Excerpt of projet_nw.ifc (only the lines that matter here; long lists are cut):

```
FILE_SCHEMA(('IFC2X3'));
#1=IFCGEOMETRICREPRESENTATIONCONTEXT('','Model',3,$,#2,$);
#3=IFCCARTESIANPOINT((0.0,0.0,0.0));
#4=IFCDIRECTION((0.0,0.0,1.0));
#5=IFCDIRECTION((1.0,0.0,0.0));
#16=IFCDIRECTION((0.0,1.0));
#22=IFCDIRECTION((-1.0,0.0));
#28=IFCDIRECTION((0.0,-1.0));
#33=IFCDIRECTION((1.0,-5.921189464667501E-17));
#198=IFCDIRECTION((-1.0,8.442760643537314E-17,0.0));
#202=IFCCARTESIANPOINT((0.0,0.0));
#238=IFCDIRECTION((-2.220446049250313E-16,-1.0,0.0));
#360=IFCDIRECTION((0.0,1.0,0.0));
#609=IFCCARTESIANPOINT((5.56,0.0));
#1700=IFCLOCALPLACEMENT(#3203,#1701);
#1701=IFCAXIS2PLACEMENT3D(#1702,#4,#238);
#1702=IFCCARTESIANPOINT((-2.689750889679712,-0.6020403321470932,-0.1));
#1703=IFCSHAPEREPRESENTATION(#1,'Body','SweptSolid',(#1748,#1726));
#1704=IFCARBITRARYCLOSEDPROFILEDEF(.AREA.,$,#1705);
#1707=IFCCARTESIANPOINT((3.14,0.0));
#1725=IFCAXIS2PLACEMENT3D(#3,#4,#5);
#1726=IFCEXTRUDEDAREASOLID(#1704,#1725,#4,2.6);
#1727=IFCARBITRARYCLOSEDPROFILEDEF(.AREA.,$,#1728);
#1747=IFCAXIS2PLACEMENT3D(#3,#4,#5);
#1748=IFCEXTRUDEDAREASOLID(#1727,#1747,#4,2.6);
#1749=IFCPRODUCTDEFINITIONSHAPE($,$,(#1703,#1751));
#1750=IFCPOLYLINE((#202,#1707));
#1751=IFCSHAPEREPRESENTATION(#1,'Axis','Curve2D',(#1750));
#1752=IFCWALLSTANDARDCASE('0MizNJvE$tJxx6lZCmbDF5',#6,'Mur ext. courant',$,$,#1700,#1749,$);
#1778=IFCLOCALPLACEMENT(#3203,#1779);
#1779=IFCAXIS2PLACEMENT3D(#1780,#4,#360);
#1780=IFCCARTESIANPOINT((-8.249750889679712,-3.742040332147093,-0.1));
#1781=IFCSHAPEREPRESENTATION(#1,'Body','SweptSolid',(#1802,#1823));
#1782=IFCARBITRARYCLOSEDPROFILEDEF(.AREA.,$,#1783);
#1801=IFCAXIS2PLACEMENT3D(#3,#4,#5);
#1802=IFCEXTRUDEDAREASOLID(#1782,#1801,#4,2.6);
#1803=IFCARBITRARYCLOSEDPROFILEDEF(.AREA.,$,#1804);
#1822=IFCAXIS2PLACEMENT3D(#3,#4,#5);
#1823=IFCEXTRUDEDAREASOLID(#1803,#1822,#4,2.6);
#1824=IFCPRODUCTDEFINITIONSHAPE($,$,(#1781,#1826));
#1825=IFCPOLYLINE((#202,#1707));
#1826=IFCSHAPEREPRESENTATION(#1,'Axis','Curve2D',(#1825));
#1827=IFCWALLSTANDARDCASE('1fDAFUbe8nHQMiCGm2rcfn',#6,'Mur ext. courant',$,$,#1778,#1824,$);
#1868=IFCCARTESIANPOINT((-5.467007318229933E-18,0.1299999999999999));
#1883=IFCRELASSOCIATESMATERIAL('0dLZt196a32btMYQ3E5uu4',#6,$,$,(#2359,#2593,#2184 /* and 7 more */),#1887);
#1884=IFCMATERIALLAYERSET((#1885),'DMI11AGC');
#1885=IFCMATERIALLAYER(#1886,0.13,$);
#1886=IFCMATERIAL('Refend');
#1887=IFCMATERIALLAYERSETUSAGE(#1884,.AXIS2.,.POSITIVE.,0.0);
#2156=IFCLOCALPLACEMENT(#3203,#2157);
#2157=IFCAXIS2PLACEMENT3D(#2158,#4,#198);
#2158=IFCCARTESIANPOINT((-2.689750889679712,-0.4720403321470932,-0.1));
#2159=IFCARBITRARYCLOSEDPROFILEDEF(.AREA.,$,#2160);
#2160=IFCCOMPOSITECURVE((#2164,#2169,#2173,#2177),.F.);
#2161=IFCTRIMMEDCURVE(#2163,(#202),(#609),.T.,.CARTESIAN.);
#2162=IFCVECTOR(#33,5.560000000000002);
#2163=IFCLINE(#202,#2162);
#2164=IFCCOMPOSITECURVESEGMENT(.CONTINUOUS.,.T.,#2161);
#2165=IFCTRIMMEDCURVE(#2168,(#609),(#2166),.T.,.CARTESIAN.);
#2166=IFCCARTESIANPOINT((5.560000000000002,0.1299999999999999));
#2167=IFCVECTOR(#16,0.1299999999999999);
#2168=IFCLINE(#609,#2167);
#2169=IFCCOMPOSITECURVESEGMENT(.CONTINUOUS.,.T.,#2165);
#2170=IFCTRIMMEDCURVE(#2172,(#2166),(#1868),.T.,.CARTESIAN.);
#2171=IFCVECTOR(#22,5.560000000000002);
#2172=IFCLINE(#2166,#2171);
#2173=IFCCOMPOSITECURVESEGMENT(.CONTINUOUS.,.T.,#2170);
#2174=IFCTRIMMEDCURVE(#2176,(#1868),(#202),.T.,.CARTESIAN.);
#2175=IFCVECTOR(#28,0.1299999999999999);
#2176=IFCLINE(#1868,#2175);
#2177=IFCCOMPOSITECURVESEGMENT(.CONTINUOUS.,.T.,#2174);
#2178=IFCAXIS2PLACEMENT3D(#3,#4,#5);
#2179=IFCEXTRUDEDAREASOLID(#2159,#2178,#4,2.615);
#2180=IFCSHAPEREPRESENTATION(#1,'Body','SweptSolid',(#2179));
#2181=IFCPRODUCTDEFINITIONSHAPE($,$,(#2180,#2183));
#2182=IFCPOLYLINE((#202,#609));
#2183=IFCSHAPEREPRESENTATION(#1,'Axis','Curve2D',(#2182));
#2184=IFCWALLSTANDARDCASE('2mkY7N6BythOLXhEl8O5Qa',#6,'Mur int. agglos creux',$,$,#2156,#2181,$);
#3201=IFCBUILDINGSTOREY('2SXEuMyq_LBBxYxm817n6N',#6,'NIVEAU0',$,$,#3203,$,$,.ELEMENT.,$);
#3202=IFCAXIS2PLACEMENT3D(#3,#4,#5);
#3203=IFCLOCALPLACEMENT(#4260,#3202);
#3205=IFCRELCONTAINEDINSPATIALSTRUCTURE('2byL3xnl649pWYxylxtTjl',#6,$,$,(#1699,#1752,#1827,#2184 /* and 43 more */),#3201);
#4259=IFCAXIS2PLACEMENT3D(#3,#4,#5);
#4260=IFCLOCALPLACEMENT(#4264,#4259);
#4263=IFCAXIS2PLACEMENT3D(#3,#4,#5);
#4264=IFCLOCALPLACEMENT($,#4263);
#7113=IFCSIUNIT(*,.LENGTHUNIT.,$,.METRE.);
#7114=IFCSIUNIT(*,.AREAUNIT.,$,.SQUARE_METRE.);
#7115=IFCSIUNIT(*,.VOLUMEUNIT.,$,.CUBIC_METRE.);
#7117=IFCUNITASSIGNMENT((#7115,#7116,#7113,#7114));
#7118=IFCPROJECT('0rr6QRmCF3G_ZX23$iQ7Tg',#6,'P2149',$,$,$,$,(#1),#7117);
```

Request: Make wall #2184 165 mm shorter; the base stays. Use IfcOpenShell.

```python
import ifcopenshell
import ifcopenshell.geom
import ifcopenshell.util.shape
import ifcopenshell.util.unit

model = ifcopenshell.open("projet_nw.ifc")
unit_scale = ifcopenshell.util.unit.calculate_unit_scale(model)
settings = ifcopenshell.geom.settings()


def volume(element):
    """Net volume in cubic metres, openings subtracted."""
    shape = ifcopenshell.geom.create_shape(settings, element)
    return ifcopenshell.util.shape.get_volume(shape.geometry)


wall = model.by_guid("2mkY7N6BythOLXhEl8O5Qa")
before = volume(wall)

body = next(r for r in wall.Representation.Representations if r.RepresentationIdentifier == "Body")
solid = body.Items[0]
old_height = solid.Depth
solid.Depth -= 0.165 / unit_scale
after = volume(wall)

print(f"height {old_height:g} -> {solid.Depth:g}, volume {before:.3f} -> {after:.3f} m3")

model.write("projet_nw-out.ifc")
```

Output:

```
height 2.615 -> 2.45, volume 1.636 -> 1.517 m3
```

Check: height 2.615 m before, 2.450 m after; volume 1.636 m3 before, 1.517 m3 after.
